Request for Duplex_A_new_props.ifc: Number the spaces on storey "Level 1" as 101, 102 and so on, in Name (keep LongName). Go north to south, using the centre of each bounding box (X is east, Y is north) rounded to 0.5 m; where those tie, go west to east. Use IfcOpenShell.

First a look at what the model holds.

```python
import ifcopenshell
import ifcopenshell.util.element
import ifcopenshell.util.placement

model = ifcopenshell.open("Duplex_A_new_props.ifc")
print(model.schema)
storey = next(s for s in model.by_type("IfcBuildingStorey") if s.Name == "Level 1")
spaces = [e for e in ifcopenshell.util.element.get_decomposition(storey) if e.is_a("IfcSpace")]
for e in sorted(spaces, key=lambda e: e.id()):
    origin = ifcopenshell.util.placement.get_local_placement(e.ObjectPlacement)[:3, 3]
    print(e.id(), e.Name, e.LongName, origin.round(2) + 0.0, sep=" | ")
```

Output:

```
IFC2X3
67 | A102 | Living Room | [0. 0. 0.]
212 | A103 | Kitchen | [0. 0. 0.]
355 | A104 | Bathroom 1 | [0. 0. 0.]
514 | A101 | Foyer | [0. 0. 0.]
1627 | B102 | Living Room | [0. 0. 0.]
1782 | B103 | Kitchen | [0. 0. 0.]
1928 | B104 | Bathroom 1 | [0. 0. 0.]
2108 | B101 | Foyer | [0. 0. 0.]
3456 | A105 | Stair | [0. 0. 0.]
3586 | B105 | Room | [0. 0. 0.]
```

```python
import ifcopenshell
import ifcopenshell.geom
import ifcopenshell.util.element
import ifcopenshell.util.shape

model = ifcopenshell.open("Duplex_A_new_props.ifc")
settings = ifcopenshell.geom.settings()
settings.set("use-world-coords", True)


def centre(element):
    shape = ifcopenshell.geom.create_shape(settings, element)
    return ifcopenshell.util.shape.get_bbox_centroid(shape.geometry)


storey = next(s for s in model.by_type("IfcBuildingStorey") if s.Name == "Level 1")
spaces = [e for e in ifcopenshell.util.element.get_decomposition(storey) if e.is_a("IfcSpace")]

# Insertion points can sit at a corner or the storey origin, so sort by the geometry (in metres).
centres = {e: centre(e) for e in spaces}
spaces.sort(key=lambda e: (-round(centres[e][1] / 0.5), centres[e][0]))

for i, e in enumerate(spaces, start=1):
    number = f"1{i:02d}"
    e.Name = number
    print(e.id(), number)

model.write("Duplex_A_new_props_v2.ifc")
```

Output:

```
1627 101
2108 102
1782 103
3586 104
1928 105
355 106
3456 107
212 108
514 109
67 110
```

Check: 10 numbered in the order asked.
